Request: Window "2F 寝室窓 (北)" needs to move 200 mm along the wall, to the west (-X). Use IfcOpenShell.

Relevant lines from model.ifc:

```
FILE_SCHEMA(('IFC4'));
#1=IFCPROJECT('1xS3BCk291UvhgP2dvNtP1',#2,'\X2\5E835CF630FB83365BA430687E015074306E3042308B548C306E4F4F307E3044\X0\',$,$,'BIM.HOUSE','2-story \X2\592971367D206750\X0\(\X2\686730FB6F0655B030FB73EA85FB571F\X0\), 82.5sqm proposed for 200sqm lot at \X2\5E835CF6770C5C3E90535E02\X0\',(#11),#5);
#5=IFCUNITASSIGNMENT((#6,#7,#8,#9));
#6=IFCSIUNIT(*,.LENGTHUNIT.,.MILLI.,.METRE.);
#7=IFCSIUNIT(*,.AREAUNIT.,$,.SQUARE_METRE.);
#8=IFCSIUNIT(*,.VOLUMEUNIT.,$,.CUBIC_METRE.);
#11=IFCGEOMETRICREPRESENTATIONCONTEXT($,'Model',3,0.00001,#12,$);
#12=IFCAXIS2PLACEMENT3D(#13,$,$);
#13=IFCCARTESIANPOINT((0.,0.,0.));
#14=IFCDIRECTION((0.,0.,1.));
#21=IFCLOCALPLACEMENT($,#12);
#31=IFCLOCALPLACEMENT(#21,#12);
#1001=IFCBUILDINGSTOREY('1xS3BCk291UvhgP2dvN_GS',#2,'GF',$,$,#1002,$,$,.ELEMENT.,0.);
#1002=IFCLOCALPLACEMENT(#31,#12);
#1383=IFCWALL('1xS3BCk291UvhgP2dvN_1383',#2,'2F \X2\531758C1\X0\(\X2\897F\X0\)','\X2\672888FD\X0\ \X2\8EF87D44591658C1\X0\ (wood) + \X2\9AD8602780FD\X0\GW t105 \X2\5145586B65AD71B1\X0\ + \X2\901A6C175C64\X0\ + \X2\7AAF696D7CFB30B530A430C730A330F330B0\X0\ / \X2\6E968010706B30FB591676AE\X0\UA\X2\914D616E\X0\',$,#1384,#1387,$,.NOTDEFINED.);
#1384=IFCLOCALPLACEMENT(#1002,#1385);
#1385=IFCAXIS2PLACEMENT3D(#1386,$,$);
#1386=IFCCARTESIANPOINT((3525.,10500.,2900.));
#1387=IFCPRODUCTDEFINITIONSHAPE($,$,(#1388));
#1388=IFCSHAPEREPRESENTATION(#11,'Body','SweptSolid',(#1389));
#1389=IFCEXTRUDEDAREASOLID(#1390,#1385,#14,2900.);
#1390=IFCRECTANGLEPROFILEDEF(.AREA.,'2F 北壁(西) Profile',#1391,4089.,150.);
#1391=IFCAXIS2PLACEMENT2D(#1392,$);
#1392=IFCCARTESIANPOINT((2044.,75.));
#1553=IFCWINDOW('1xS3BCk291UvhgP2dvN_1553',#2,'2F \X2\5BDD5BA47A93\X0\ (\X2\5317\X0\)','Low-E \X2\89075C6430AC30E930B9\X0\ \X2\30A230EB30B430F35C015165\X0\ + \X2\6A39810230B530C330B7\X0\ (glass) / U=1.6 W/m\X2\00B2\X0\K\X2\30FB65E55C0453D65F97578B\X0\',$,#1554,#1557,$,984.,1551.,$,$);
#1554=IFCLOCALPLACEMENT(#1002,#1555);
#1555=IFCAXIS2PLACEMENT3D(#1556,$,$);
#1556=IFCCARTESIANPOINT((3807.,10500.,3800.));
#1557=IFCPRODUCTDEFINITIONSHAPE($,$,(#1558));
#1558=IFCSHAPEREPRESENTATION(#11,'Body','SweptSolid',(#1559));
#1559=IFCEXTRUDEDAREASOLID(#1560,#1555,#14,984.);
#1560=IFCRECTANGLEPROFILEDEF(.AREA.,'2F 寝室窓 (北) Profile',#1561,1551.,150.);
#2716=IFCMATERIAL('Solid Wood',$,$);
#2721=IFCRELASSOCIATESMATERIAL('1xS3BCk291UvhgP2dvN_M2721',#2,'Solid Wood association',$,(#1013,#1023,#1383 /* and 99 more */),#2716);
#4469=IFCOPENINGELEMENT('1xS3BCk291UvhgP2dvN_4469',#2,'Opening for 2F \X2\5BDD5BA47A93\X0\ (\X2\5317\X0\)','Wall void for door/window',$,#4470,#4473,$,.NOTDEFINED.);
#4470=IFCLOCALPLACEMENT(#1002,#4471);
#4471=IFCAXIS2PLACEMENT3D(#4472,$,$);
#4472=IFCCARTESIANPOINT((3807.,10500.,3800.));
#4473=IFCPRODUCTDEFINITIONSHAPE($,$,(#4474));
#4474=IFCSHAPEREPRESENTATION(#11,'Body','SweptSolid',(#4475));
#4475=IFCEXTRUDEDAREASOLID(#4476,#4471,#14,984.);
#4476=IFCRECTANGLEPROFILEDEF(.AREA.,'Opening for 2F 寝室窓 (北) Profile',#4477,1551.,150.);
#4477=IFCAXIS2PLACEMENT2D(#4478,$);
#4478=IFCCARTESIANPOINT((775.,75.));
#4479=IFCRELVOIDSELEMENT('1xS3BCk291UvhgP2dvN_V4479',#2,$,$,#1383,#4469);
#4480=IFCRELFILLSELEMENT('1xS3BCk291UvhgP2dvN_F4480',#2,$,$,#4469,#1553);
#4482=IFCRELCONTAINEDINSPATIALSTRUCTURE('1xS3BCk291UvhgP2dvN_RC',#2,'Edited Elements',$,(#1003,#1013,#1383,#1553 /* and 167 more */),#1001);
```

```python
import ifcopenshell
import ifcopenshell.api.geometry
import ifcopenshell.util.placement
import ifcopenshell.util.unit

model = ifcopenshell.open("model.ifc")
unit_scale = ifcopenshell.util.unit.calculate_unit_scale(model)

window = model.by_guid("1xS3BCk291UvhgP2dvN_1553")
opening = window.FillsVoids[0].RelatingOpeningElement
wall = opening.VoidsElements[0].RelatingBuildingElement

wall_matrix = ifcopenshell.util.placement.get_local_placement(wall.ObjectPlacement)
shift = wall_matrix[:3, 0] * -0.2 / unit_scale
before = ifcopenshell.util.placement.get_local_placement(window.ObjectPlacement)[:3, 3].copy()

# The window is not placed relative to its opening, so move both.
for product in (opening, window):
    matrix = ifcopenshell.util.placement.get_local_placement(product.ObjectPlacement)
    matrix[:3, 3] += shift
    ifcopenshell.api.geometry.edit_object_placement(model, product=product, matrix=matrix, is_si=False)

after = ifcopenshell.util.placement.get_local_placement(window.ObjectPlacement)[:3, 3]
print("window moved by", (after - before).round(3) + 0.0)

model.write("model-out.ifc")
```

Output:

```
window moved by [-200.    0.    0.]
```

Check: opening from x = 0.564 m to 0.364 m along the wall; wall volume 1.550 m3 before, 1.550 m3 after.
